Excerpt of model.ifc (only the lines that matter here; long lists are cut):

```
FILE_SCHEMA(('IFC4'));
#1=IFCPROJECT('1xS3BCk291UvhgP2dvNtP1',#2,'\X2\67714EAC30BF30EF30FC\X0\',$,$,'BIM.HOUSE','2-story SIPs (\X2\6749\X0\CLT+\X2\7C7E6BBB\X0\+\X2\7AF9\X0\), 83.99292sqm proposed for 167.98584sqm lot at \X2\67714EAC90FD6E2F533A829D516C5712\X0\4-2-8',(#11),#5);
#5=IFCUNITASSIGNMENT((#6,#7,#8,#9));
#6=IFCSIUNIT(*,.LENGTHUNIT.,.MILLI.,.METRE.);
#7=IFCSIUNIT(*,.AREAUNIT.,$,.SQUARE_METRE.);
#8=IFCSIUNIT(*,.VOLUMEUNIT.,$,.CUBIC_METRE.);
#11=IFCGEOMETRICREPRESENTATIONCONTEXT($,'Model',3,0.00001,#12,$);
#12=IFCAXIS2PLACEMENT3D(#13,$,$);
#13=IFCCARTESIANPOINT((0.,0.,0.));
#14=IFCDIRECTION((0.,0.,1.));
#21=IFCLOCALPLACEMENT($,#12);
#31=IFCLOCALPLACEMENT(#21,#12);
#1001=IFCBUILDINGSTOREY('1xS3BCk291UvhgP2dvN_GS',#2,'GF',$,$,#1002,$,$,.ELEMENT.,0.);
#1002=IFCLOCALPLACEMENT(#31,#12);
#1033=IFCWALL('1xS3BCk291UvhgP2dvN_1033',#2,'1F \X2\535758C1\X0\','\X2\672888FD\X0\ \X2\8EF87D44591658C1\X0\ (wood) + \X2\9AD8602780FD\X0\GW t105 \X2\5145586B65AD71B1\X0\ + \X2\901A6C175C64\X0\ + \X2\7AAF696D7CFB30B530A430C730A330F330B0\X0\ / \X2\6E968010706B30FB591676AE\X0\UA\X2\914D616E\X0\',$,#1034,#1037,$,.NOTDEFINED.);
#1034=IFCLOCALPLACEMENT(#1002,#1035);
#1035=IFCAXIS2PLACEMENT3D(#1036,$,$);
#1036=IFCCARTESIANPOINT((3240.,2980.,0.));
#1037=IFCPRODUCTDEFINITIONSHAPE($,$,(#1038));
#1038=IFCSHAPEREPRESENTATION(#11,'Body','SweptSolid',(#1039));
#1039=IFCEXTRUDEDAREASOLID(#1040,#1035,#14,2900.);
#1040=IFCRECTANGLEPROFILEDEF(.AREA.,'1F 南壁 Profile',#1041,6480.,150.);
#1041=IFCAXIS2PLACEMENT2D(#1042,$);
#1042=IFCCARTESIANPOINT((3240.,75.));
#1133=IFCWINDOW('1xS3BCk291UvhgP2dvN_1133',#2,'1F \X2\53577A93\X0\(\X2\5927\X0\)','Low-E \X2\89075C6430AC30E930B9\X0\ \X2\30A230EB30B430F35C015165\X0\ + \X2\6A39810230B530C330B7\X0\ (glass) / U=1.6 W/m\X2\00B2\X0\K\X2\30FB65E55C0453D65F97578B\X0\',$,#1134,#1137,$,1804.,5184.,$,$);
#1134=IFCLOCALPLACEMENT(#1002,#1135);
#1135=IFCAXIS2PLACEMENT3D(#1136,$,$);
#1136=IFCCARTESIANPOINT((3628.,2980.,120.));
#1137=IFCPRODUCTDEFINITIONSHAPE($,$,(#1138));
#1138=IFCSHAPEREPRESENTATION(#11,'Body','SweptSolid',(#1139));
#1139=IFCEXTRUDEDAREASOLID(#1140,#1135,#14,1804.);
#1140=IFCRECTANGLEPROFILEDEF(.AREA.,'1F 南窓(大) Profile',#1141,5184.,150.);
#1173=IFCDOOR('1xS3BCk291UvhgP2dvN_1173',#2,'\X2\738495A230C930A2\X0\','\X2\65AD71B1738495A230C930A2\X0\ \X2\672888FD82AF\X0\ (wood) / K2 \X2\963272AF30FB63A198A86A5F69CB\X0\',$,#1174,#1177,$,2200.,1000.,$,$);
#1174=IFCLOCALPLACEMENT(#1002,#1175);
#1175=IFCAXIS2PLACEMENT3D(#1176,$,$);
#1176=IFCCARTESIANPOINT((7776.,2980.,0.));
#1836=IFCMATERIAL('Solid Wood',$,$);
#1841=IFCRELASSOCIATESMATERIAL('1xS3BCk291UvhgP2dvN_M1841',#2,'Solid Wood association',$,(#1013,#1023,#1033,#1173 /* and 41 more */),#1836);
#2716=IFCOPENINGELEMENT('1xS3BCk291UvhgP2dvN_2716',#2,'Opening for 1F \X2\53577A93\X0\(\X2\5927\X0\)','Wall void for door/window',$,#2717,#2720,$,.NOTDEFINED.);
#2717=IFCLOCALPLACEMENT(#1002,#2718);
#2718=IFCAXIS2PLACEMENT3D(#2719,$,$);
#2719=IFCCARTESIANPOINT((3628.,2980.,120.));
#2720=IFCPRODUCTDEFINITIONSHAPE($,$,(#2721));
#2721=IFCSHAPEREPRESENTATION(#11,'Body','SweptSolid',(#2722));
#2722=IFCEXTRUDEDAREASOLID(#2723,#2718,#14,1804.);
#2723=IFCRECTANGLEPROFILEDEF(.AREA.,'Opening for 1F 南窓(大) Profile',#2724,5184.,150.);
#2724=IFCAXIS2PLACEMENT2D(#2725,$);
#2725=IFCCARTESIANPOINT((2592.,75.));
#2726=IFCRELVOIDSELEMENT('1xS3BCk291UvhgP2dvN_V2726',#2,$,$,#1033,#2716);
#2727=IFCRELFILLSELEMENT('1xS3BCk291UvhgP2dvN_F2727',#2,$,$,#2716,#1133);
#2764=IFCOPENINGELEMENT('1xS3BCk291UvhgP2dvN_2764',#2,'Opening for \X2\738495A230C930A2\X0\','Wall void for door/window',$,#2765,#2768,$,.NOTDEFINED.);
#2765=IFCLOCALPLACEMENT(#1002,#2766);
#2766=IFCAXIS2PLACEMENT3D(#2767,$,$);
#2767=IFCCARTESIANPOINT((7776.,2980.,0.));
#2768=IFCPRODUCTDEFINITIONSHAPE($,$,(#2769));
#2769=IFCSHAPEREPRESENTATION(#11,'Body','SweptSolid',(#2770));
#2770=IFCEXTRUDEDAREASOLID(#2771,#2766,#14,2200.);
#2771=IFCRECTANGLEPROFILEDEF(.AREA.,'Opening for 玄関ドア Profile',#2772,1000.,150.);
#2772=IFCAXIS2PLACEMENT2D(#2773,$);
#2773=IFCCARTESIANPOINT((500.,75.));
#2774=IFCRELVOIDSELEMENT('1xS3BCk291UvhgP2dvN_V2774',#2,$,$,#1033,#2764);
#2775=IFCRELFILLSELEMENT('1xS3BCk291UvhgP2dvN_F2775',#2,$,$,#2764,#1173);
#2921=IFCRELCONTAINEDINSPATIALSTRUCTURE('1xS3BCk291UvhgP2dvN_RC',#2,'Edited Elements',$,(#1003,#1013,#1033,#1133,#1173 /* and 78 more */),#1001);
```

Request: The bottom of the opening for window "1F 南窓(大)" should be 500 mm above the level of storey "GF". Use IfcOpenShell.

```python
import numpy as np
import ifcopenshell
import ifcopenshell.api.geometry
import ifcopenshell.geom
import ifcopenshell.util.element
import ifcopenshell.util.placement
import ifcopenshell.util.shape
import ifcopenshell.util.unit

model = ifcopenshell.open("model.ifc")
unit_scale = ifcopenshell.util.unit.calculate_unit_scale(model)

window = model.by_guid("1xS3BCk291UvhgP2dvN_1133")
opening = window.FillsVoids[0].RelatingOpeningElement
storey = ifcopenshell.util.element.get_container(window, ifc_class="IfcBuildingStorey")
level = ifcopenshell.util.placement.get_local_placement(storey.ObjectPlacement)[2, 3]

# The opening's origin need not be at the sill, so measure its lowest point.
shape = ifcopenshell.geom.create_shape(ifcopenshell.geom.settings(), opening)
bottom = ifcopenshell.util.shape.get_shape_bottom_elevation(shape, shape.geometry) / unit_scale
dz = level + 500.0 - bottom

shift = np.array([0.0, 0.0, dz])
# The window is not placed relative to its opening, so move both.
for product in (opening, window):
    matrix = ifcopenshell.util.placement.get_local_placement(product.ObjectPlacement)
    matrix[:3, 3] += shift
    ifcopenshell.api.geometry.edit_object_placement(model, product=product, matrix=matrix, is_si=False)

print(f"moved by {dz * unit_scale:+.3f} m")

model.write("model-out.ifc")
```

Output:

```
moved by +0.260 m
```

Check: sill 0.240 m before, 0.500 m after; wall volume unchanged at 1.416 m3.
